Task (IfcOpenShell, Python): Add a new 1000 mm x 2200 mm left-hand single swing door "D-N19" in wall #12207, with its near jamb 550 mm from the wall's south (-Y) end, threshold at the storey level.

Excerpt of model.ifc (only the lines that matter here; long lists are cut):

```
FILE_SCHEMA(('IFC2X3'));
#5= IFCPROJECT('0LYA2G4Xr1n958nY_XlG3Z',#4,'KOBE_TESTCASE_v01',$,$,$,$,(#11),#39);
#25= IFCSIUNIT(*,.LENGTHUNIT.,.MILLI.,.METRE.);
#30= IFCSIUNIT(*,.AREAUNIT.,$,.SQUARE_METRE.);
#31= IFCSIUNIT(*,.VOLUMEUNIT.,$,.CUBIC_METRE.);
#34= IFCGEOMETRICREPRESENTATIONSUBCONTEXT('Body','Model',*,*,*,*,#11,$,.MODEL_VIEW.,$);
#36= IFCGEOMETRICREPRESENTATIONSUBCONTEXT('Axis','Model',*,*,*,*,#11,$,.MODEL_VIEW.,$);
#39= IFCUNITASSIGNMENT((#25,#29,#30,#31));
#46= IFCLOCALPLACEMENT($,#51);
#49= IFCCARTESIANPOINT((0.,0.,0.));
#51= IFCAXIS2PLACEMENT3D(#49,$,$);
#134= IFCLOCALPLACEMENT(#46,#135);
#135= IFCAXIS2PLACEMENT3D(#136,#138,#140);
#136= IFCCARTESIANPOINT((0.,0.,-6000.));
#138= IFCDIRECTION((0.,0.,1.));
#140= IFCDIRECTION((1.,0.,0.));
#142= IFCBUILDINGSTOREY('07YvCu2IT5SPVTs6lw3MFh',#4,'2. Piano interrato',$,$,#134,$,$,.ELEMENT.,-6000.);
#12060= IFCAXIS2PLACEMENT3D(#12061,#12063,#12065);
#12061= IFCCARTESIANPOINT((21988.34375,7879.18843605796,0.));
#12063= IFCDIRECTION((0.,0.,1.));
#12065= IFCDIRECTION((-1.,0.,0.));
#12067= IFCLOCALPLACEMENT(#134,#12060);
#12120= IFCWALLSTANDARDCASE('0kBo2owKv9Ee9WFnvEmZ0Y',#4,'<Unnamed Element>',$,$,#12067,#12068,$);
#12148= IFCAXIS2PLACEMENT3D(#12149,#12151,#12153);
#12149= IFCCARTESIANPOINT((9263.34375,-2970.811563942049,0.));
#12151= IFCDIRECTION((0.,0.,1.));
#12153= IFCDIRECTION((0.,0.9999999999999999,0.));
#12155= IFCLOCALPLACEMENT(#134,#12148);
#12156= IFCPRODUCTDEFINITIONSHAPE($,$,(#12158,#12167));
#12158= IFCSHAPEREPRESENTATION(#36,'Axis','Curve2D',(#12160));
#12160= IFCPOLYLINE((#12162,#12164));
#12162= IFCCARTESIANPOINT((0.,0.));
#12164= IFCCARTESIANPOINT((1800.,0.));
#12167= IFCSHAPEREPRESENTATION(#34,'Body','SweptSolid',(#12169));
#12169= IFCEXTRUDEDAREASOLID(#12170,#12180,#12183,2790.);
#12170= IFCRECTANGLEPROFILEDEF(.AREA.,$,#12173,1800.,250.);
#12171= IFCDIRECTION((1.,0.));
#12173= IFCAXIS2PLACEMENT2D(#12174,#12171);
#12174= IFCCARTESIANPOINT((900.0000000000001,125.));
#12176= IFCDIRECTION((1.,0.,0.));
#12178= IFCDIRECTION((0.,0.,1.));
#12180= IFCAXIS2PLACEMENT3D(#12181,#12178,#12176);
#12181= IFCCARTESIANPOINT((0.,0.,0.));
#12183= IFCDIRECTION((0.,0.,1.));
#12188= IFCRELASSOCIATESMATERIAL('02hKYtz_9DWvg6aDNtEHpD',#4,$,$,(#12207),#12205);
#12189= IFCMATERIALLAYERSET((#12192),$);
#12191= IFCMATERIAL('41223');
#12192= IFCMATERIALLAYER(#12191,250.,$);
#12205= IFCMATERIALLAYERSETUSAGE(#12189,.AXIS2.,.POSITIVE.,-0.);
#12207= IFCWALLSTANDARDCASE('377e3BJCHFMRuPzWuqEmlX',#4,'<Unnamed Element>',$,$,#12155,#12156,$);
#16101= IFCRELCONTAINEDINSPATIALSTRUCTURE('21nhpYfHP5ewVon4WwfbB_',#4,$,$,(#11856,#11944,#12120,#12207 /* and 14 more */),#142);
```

```python
import numpy as np
import ifcopenshell
import ifcopenshell.api.feature
import ifcopenshell.api.geometry
import ifcopenshell.api.root
import ifcopenshell.api.spatial
import ifcopenshell.api.type
import ifcopenshell.geom
import ifcopenshell.util.element
import ifcopenshell.util.placement
import ifcopenshell.util.representation
import ifcopenshell.util.shape
import ifcopenshell.util.unit

model = ifcopenshell.open("model.ifc")
unit_scale = ifcopenshell.util.unit.calculate_unit_scale(model)
settings = ifcopenshell.geom.settings()


def volume(element):
    """Net volume in cubic metres, openings subtracted."""
    shape = ifcopenshell.geom.create_shape(settings, element)
    return ifcopenshell.util.shape.get_volume(shape.geometry)


wall = model.by_guid("377e3BJCHFMRuPzWuqEmlX")
storey = ifcopenshell.util.element.get_container(wall, ifc_class="IfcBuildingStorey")
context = ifcopenshell.util.representation.get_context(model, "Model", "Body", "MODEL_VIEW")
before = volume(wall)

width, height, from_end, sill = 1, 2.2, 0.55, 0.0  # metres

# The wall runs along its own X axis, and the end named is its -X end.
wall_shape = ifcopenshell.geom.create_shape(settings, wall)
x, y, z = ifcopenshell.util.shape.get_vertices(wall_shape.geometry).T
start = x.min() + from_end
face, thickness = float(y.min()), float(y.max() - y.min())
wall_matrix = ifcopenshell.util.placement.get_local_placement(wall.ObjectPlacement)
level = ifcopenshell.util.placement.get_local_placement(storey.ObjectPlacement)[2, 3]


def in_wall(x, y):
    """Placement at x, y metres in the wall's axes, at sill height."""
    matrix = wall_matrix.copy()
    matrix[:, 3] = wall_matrix @ np.array([x / unit_scale, y / unit_scale, 0.0, 1.0])
    matrix[2, 3] = level + sill / unit_scale
    return matrix


# Opening: a box that overshoots both wall faces by 50 mm.
opening = ifcopenshell.api.root.create_entity(model, ifc_class="IfcOpeningElement")
box = ifcopenshell.api.geometry.add_wall_representation(
    model, context=context, length=width, height=height, thickness=thickness + 0.1
)
ifcopenshell.api.geometry.assign_representation(model, product=opening, representation=box)
ifcopenshell.api.geometry.edit_object_placement(model, product=opening, matrix=in_wall(start, face - 0.05), is_si=False)
ifcopenshell.api.feature.add_feature(model, feature=opening, element=wall)

door = ifcopenshell.api.root.create_entity(model, ifc_class="IfcDoor", name="D-N19")
door.OverallWidth, door.OverallHeight = width / unit_scale, height / unit_scale
body = ifcopenshell.api.geometry.add_door_representation(
    model,
    context=context,
    overall_width=door.OverallWidth,
    overall_height=door.OverallHeight,
    operation_type="SINGLE_SWING_LEFT",
    lining_properties={"LiningDepth": thickness / unit_scale, "ThresholdDepth": thickness / unit_scale},
)
ifcopenshell.api.geometry.assign_representation(model, product=door, representation=body)
ifcopenshell.api.spatial.assign_container(model, products=[door], relating_structure=storey)
fills = ifcopenshell.api.feature.add_filling(model, opening=opening, element=door)
fills.OwnerHistory = door.OwnerHistory  # required in IFC2X3

# IFC2X3 keeps the operation on the door style.
style = ifcopenshell.api.root.create_entity(model, ifc_class="IfcDoorStyle", name="D-N19")
style.OperationType, style.ConstructionType = "SINGLE_SWING_LEFT", "NOTDEFINED"
style.ParameterTakesPrecedence = style.Sizeable = False
ifcopenshell.api.type.assign_type(model, related_objects=[door], relating_type=style)

# The lining spans the wall, so the door starts at the wall face.
ifcopenshell.api.geometry.edit_object_placement(model, product=door, matrix=in_wall(start, face), is_si=False)

after = volume(wall)

print(f"wall volume {before:.3f} -> {after:.3f} m3")

model.write("model-out.ifc")
```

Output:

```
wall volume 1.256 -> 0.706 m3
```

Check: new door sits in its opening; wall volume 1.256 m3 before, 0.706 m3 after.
